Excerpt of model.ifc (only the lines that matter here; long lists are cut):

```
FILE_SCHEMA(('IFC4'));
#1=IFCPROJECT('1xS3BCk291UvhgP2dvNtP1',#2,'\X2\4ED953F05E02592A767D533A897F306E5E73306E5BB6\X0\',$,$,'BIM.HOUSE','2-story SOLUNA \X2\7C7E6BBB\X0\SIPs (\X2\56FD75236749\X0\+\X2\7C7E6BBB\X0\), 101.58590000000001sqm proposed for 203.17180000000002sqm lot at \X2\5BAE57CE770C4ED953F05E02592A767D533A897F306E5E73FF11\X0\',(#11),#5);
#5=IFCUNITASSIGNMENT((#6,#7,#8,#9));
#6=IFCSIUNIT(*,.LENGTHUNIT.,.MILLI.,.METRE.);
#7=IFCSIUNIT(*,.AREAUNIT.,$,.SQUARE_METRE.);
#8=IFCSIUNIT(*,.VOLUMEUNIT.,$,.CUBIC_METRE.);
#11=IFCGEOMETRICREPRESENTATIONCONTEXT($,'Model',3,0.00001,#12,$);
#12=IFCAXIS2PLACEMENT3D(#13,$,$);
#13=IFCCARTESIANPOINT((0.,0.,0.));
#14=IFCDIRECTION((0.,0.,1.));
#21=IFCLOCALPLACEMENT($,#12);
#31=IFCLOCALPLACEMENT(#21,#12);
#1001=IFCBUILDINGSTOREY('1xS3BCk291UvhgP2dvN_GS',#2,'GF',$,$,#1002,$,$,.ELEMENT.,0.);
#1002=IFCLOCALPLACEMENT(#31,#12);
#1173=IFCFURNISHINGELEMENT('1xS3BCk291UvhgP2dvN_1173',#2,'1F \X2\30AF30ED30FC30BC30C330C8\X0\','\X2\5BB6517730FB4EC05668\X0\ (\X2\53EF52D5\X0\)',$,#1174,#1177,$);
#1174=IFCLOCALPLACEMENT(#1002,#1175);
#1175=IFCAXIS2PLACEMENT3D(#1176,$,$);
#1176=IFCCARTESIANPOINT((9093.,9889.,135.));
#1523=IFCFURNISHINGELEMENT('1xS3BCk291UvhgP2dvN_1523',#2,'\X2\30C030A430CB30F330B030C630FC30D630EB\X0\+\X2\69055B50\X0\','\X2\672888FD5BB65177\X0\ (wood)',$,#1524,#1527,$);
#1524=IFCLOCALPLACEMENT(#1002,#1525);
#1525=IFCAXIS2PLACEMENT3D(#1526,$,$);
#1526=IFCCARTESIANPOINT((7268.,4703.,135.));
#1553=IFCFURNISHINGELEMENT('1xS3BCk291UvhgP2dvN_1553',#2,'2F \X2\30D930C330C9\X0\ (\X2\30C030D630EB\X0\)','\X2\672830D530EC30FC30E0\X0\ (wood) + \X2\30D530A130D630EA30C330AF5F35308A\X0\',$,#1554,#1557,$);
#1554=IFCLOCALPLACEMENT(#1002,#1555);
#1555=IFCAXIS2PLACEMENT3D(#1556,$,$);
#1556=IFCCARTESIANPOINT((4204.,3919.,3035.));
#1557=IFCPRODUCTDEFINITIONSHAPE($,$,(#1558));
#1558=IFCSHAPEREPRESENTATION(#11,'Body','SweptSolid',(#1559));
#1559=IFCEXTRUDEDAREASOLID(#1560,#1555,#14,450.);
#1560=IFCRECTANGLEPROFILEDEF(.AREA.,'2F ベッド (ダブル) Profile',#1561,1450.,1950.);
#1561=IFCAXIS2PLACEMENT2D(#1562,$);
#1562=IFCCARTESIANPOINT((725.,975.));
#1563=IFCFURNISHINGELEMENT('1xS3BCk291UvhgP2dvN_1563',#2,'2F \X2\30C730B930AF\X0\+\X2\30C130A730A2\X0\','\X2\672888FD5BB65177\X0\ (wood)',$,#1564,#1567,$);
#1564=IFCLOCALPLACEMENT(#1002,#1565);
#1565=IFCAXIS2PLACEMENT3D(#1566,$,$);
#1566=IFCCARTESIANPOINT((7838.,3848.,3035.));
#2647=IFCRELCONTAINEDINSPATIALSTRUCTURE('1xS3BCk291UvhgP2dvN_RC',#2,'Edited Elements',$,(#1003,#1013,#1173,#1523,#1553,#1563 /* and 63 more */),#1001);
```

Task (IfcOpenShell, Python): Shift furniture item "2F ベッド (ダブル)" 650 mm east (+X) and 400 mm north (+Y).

```python
import ifcopenshell
import ifcopenshell.api.geometry
import ifcopenshell.util.placement
import ifcopenshell.util.unit

model = ifcopenshell.open("model.ifc")
unit_scale = ifcopenshell.util.unit.calculate_unit_scale(model)

item = model.by_id(1553)
matrix = ifcopenshell.util.placement.get_local_placement(item.ObjectPlacement)
matrix[0, 3] += 0.65 / unit_scale
matrix[1, 3] += 0.4 / unit_scale
ifcopenshell.api.geometry.edit_object_placement(model, product=item, matrix=matrix, is_si=False)

print(ifcopenshell.util.placement.get_local_placement(item.ObjectPlacement).round(3) + 0.0)

model.write("model_updated.ifc")
```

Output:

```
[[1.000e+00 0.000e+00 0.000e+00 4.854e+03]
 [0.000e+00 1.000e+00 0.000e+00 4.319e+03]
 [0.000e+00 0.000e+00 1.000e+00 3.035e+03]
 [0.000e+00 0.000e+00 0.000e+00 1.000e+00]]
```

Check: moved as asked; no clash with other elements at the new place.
